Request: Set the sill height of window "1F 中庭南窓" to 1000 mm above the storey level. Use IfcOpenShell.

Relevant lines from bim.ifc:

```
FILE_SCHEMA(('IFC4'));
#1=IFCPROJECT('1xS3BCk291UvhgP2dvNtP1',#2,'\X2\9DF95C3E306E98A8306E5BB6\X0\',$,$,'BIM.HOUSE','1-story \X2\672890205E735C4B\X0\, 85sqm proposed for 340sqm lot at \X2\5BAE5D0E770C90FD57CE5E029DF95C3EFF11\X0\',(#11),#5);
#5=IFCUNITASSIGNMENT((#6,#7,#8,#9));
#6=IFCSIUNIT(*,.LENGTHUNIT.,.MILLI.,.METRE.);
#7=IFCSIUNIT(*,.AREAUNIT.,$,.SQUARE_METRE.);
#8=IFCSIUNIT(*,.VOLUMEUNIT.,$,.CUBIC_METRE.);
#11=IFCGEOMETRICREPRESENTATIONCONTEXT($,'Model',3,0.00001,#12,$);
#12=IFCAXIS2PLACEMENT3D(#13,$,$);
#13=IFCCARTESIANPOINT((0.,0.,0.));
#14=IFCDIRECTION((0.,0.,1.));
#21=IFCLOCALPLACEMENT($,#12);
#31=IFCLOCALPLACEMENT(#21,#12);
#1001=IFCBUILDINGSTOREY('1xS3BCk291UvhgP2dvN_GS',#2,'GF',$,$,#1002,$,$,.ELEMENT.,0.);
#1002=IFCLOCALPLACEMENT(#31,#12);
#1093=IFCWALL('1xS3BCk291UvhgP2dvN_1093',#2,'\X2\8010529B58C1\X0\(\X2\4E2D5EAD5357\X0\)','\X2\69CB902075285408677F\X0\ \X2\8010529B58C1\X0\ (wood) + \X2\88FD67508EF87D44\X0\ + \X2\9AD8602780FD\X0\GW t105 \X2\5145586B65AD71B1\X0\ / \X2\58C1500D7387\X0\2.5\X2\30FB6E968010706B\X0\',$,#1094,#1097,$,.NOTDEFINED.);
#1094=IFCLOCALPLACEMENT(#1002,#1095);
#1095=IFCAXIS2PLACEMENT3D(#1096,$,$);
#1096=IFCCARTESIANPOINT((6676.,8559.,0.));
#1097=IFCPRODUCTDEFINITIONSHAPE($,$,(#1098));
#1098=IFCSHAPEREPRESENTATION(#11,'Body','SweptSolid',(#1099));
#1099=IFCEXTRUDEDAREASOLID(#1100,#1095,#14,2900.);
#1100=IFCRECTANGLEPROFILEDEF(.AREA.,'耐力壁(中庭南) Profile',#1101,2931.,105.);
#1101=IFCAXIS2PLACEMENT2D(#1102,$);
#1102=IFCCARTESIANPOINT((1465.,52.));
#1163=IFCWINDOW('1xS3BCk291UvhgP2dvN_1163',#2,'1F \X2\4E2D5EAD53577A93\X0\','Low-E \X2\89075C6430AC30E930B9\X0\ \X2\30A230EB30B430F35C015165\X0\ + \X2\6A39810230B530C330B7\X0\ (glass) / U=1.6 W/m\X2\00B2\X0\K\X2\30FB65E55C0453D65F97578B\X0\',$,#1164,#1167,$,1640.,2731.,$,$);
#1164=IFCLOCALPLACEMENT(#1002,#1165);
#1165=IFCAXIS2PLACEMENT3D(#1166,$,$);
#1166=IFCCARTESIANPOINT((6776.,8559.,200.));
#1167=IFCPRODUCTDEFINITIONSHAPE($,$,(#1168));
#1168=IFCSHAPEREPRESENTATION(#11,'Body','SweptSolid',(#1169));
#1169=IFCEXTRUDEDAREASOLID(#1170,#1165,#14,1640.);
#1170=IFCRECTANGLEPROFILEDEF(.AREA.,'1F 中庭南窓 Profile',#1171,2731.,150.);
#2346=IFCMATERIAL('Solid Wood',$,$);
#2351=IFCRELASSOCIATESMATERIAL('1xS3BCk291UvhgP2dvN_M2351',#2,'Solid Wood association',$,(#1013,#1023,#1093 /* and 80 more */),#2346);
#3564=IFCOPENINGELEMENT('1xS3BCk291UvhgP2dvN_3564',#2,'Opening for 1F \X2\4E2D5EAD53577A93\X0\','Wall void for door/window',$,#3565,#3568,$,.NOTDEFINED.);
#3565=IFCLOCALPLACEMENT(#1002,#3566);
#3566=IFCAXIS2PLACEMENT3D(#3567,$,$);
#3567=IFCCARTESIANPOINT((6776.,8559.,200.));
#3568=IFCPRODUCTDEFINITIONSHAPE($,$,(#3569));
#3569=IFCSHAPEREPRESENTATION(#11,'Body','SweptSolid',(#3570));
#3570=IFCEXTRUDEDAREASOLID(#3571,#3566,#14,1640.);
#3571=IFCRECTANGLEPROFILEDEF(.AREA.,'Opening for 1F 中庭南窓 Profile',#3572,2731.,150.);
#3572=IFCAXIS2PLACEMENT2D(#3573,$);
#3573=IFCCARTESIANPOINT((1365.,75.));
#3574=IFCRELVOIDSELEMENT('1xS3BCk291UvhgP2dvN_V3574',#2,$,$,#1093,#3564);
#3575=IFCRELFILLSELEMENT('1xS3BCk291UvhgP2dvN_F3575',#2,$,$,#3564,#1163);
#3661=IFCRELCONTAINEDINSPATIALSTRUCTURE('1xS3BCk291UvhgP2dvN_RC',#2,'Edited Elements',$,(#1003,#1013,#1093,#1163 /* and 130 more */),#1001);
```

```python
import numpy as np
import ifcopenshell
import ifcopenshell.api.geometry
import ifcopenshell.geom
import ifcopenshell.util.element
import ifcopenshell.util.placement
import ifcopenshell.util.shape
import ifcopenshell.util.unit

model = ifcopenshell.open("bim.ifc")
unit_scale = ifcopenshell.util.unit.calculate_unit_scale(model)

window = model.by_guid("1xS3BCk291UvhgP2dvN_1163")
opening = window.FillsVoids[0].RelatingOpeningElement
storey = ifcopenshell.util.element.get_container(window, ifc_class="IfcBuildingStorey")
level = ifcopenshell.util.placement.get_local_placement(storey.ObjectPlacement)[2, 3]

# The opening's origin need not be at the sill, so measure its lowest point.
shape = ifcopenshell.geom.create_shape(ifcopenshell.geom.settings(), opening)
bottom = ifcopenshell.util.shape.get_shape_bottom_elevation(shape, shape.geometry) / unit_scale
dz = level + 1 / unit_scale - bottom

shift = np.array([0.0, 0.0, dz])
# The window is not placed relative to its opening, so move both.
for product in (opening, window):
    matrix = ifcopenshell.util.placement.get_local_placement(product.ObjectPlacement)
    matrix[:3, 3] += shift
    ifcopenshell.api.geometry.edit_object_placement(model, product=product, matrix=matrix, is_si=False)

print(f"moved by {dz * unit_scale:+.3f} m")

model.write("bim_v2.ifc")
```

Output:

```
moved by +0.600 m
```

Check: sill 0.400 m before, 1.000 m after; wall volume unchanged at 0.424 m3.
